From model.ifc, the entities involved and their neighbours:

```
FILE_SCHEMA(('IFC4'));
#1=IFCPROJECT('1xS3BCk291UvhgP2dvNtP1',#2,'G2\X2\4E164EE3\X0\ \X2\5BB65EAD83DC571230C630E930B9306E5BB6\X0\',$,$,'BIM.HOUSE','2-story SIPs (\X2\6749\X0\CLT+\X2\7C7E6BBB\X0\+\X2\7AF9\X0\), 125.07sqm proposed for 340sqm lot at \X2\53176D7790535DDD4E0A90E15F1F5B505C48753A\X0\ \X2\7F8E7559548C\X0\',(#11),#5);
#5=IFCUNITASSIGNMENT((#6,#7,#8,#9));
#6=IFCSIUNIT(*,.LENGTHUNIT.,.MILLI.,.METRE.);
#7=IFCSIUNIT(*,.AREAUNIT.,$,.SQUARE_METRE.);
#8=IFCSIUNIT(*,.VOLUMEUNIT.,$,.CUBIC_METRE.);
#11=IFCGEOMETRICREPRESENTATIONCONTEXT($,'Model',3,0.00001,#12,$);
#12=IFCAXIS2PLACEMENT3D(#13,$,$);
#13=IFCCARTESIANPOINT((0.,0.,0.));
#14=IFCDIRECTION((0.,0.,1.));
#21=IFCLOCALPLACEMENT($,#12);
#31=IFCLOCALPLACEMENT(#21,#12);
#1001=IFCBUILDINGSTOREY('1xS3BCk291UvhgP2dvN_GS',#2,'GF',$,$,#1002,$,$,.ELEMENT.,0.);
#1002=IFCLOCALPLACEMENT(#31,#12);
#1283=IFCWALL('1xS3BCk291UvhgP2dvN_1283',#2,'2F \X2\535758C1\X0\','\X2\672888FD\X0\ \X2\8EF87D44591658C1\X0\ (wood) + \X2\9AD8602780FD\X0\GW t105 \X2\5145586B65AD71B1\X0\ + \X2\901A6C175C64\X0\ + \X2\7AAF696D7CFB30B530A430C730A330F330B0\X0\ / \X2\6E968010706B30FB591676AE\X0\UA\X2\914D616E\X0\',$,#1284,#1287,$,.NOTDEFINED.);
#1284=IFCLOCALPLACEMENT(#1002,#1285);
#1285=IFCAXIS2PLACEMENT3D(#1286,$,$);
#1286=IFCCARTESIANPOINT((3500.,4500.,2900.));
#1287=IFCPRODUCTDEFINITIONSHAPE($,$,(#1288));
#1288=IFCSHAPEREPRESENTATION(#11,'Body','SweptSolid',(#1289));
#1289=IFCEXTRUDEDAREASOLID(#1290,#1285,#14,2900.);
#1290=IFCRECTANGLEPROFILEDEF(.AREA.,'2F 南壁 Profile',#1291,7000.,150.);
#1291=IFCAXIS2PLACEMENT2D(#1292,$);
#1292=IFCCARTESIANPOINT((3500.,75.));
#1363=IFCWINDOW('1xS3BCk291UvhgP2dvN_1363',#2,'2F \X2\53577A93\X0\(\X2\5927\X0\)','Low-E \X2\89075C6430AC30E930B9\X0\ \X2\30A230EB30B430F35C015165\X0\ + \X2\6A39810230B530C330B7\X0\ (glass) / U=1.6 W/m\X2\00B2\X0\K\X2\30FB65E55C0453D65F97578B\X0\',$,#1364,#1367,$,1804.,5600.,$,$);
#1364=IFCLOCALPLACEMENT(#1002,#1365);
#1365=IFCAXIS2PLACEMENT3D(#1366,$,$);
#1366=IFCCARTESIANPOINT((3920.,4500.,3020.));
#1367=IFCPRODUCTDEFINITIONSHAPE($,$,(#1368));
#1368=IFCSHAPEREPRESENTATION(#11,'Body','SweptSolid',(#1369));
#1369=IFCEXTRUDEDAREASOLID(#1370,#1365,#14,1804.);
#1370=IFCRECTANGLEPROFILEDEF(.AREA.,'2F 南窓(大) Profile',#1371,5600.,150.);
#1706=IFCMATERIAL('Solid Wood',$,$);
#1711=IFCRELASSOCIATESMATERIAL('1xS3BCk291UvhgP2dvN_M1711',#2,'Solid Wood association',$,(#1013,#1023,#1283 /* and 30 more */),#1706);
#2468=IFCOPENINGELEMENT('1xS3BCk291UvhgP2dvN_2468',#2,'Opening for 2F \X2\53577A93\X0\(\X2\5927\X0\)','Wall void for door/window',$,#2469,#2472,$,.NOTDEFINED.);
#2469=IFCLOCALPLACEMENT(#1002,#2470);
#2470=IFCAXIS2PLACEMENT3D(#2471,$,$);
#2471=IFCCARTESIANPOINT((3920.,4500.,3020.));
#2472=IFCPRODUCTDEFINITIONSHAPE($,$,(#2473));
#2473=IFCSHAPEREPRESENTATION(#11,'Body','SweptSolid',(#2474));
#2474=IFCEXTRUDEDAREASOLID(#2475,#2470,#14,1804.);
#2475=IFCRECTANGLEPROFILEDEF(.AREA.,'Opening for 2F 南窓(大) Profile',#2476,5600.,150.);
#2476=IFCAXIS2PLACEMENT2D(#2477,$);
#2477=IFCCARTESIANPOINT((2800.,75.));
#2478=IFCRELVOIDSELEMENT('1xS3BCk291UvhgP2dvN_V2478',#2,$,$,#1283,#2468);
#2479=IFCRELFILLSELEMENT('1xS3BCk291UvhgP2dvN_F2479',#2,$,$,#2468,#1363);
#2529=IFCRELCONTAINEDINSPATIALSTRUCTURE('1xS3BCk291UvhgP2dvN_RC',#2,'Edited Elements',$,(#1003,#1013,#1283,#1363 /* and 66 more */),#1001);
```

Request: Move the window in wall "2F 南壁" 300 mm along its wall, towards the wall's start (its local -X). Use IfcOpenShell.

```python
import ifcopenshell
import ifcopenshell.api.geometry
import ifcopenshell.util.placement
import ifcopenshell.util.unit

model = ifcopenshell.open("model.ifc")
unit_scale = ifcopenshell.util.unit.calculate_unit_scale(model)

window = model.by_id(1363)
opening = window.FillsVoids[0].RelatingOpeningElement
wall = opening.VoidsElements[0].RelatingBuildingElement

wall_matrix = ifcopenshell.util.placement.get_local_placement(wall.ObjectPlacement)
shift = wall_matrix[:3, 0] * -0.3 / unit_scale
before = ifcopenshell.util.placement.get_local_placement(window.ObjectPlacement)[:3, 3].copy()

# The window is not placed relative to its opening, so move both.
for product in (opening, window):
    matrix = ifcopenshell.util.placement.get_local_placement(product.ObjectPlacement)
    matrix[:3, 3] += shift
    ifcopenshell.api.geometry.edit_object_placement(model, product=product, matrix=matrix, is_si=False)

after = ifcopenshell.util.placement.get_local_placement(window.ObjectPlacement)[:3, 3]
print("window moved by", (after - before).round(3) + 0.0)

model.write("model_updated.ifc")
```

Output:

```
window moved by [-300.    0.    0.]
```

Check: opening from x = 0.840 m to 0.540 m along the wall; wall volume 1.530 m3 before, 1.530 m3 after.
